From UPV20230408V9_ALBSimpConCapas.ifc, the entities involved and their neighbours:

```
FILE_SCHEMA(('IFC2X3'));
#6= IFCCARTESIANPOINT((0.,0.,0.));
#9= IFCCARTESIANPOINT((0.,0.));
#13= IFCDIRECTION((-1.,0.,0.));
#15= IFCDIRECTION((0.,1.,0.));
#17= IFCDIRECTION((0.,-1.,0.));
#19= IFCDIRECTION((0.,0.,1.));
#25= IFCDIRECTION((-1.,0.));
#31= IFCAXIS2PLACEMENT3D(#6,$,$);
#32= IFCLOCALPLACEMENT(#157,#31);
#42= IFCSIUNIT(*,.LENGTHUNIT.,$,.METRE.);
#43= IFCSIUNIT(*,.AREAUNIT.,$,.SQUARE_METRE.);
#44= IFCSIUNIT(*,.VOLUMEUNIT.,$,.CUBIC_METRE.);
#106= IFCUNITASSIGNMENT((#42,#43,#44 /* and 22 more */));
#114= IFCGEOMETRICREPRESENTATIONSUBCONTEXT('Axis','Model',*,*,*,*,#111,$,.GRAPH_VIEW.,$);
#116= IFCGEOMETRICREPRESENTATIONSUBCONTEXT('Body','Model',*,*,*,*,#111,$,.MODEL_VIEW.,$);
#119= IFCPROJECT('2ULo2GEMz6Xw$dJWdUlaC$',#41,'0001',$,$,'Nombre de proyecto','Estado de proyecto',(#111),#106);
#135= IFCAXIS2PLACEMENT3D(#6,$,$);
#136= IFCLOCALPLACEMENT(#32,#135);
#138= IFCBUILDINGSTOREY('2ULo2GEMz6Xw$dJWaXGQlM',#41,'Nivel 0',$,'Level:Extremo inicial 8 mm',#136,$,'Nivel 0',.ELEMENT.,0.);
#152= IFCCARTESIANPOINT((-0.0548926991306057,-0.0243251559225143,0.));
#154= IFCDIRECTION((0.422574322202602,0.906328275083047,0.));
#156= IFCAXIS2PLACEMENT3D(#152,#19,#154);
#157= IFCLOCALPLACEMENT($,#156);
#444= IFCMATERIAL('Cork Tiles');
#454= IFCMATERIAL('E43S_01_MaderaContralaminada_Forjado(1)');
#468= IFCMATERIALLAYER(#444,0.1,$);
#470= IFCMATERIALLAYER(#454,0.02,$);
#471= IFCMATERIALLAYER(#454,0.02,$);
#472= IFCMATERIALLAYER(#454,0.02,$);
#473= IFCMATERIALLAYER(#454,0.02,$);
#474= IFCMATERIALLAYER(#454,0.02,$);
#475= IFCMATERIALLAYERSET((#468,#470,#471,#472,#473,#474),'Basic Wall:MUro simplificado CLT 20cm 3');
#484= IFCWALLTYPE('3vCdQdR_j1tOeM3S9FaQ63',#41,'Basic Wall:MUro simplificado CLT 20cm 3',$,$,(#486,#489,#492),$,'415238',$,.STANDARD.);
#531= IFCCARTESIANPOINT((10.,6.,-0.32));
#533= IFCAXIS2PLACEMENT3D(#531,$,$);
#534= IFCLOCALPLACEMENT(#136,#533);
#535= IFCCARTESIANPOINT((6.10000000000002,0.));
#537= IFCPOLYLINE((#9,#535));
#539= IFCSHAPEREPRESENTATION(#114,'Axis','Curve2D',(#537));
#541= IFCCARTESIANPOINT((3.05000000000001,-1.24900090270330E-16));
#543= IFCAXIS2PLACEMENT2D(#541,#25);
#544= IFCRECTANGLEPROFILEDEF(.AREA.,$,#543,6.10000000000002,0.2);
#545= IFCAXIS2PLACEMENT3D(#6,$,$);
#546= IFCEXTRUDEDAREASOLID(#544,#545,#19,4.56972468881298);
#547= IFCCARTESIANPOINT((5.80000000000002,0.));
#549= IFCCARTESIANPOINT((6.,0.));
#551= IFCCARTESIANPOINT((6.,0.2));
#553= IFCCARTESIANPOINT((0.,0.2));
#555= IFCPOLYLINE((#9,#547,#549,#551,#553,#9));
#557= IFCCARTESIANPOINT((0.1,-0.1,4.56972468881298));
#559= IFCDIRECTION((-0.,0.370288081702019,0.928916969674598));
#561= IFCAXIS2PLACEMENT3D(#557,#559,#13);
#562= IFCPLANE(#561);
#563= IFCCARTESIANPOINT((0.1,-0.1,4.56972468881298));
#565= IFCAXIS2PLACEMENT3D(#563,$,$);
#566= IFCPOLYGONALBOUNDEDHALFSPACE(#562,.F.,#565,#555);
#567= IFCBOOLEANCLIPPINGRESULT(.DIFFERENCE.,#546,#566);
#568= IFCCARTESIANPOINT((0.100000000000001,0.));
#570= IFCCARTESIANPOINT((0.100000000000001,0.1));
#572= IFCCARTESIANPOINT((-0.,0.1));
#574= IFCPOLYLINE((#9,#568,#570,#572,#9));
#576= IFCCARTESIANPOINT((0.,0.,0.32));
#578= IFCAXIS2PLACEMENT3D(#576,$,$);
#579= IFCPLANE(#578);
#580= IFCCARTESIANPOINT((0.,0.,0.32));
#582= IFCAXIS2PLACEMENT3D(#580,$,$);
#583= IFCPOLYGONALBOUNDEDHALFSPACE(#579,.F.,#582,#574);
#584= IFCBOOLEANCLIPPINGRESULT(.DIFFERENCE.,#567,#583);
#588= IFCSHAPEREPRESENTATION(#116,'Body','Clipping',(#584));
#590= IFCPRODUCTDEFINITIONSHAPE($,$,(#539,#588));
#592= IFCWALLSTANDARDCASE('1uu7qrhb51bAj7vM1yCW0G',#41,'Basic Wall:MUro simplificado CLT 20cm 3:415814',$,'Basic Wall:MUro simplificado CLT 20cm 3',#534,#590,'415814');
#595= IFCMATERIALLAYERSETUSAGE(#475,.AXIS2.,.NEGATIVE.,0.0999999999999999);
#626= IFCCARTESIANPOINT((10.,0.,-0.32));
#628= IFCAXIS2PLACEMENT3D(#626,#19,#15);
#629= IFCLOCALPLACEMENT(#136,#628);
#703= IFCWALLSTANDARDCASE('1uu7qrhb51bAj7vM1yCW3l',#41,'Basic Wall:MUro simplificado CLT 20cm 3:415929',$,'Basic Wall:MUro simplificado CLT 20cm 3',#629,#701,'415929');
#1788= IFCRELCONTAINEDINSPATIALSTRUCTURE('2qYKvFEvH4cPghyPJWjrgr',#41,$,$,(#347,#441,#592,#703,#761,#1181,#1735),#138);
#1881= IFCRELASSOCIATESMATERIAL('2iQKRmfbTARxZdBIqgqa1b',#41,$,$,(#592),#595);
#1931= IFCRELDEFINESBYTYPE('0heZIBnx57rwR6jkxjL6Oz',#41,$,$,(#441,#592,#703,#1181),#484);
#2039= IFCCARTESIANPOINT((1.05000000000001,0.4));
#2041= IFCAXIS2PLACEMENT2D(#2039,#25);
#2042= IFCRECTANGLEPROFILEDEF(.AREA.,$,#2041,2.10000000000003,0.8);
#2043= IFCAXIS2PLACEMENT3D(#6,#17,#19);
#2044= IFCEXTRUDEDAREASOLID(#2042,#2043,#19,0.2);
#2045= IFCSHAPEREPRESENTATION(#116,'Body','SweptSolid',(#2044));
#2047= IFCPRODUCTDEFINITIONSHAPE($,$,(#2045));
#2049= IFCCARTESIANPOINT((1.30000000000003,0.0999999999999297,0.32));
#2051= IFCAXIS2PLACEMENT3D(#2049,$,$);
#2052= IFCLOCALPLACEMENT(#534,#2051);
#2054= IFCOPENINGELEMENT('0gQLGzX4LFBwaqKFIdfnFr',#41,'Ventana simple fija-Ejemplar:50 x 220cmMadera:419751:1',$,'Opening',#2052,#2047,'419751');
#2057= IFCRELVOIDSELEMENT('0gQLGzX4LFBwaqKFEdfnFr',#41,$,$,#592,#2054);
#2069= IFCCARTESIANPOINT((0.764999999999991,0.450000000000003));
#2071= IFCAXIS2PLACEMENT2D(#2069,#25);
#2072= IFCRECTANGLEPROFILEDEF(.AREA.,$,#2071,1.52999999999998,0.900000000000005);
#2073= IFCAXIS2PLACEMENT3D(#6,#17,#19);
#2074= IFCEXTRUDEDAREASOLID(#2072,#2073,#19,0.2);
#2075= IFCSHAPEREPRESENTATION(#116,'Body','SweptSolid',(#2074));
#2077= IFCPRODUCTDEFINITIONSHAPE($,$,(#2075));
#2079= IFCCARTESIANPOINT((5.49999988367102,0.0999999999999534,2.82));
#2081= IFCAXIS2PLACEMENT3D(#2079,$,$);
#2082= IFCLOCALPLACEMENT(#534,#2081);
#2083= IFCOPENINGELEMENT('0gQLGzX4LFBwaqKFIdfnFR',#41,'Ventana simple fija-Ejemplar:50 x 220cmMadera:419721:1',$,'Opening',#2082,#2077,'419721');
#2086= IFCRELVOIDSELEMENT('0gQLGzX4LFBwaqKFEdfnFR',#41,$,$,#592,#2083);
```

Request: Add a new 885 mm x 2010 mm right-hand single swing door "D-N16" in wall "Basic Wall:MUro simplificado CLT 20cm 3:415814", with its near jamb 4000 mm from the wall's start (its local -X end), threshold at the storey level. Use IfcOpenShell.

```python
import numpy as np
import ifcopenshell
import ifcopenshell.api.feature
import ifcopenshell.api.geometry
import ifcopenshell.api.root
import ifcopenshell.api.spatial
import ifcopenshell.api.type
import ifcopenshell.geom
import ifcopenshell.util.element
import ifcopenshell.util.placement
import ifcopenshell.util.representation
import ifcopenshell.util.shape
import ifcopenshell.util.unit

model = ifcopenshell.open("UPV20230408V9_ALBSimpConCapas.ifc")
unit_scale = ifcopenshell.util.unit.calculate_unit_scale(model)
settings = ifcopenshell.geom.settings()


def volume(element):
    """Net volume in cubic metres, openings subtracted."""
    shape = ifcopenshell.geom.create_shape(settings, element)
    return ifcopenshell.util.shape.get_volume(shape.geometry)


wall = model.by_guid("1uu7qrhb51bAj7vM1yCW0G")
storey = ifcopenshell.util.element.get_container(wall, ifc_class="IfcBuildingStorey")
context = ifcopenshell.util.representation.get_context(model, "Model", "Body", "MODEL_VIEW")
before = volume(wall)

width, height, from_end, sill = 0.885, 2.01, 4, 0.0  # metres

# The wall runs along its own X axis, and the end named is its -X end.
wall_shape = ifcopenshell.geom.create_shape(settings, wall)
x, y, z = ifcopenshell.util.shape.get_vertices(wall_shape.geometry).T
start = x.min() + from_end
face, thickness = float(y.min()), float(y.max() - y.min())
wall_matrix = ifcopenshell.util.placement.get_local_placement(wall.ObjectPlacement)
level = ifcopenshell.util.placement.get_local_placement(storey.ObjectPlacement)[2, 3]


def in_wall(x, y):
    """Placement at x, y metres in the wall's axes, at sill height."""
    matrix = wall_matrix.copy()
    matrix[:, 3] = wall_matrix @ np.array([x / unit_scale, y / unit_scale, 0.0, 1.0])
    matrix[2, 3] = level + sill / unit_scale
    return matrix


# Opening: a box that overshoots both wall faces by 50 mm.
opening = ifcopenshell.api.root.create_entity(model, ifc_class="IfcOpeningElement")
box = ifcopenshell.api.geometry.add_wall_representation(
    model, context=context, length=width, height=height, thickness=thickness + 0.1
)
ifcopenshell.api.geometry.assign_representation(model, product=opening, representation=box)
ifcopenshell.api.geometry.edit_object_placement(model, product=opening, matrix=in_wall(start, face - 0.05), is_si=False)
ifcopenshell.api.feature.add_feature(model, feature=opening, element=wall)

door = ifcopenshell.api.root.create_entity(model, ifc_class="IfcDoor", name="D-N16")
door.OverallWidth, door.OverallHeight = width / unit_scale, height / unit_scale
body = ifcopenshell.api.geometry.add_door_representation(
    model,
    context=context,
    overall_width=door.OverallWidth,
    overall_height=door.OverallHeight,
    operation_type="SINGLE_SWING_RIGHT",
    lining_properties={"LiningDepth": thickness / unit_scale, "ThresholdDepth": thickness / unit_scale},
)
ifcopenshell.api.geometry.assign_representation(model, product=door, representation=body)
ifcopenshell.api.spatial.assign_container(model, products=[door], relating_structure=storey)
fills = ifcopenshell.api.feature.add_filling(model, opening=opening, element=door)
fills.OwnerHistory = door.OwnerHistory  # required in IFC2X3

# IFC2X3 keeps the operation on the door style.
style = ifcopenshell.api.root.create_entity(model, ifc_class="IfcDoorStyle", name="D-N16")
style.OperationType, style.ConstructionType = "SINGLE_SWING_RIGHT", "NOTDEFINED"
style.ParameterTakesPrecedence = style.Sizeable = False
ifcopenshell.api.type.assign_type(model, related_objects=[door], relating_type=style)

# The lining spans the wall, so the door starts at the wall face.
ifcopenshell.api.geometry.edit_object_placement(model, product=door, matrix=in_wall(start, face), is_si=False)

after = volume(wall)

print(f"wall volume {before:.3f} -> {after:.3f} m3")

model.write("UPV20230408V9_ALBSimpConCapas_rev.ifc")
```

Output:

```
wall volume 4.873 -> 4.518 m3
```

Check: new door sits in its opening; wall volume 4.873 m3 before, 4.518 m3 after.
